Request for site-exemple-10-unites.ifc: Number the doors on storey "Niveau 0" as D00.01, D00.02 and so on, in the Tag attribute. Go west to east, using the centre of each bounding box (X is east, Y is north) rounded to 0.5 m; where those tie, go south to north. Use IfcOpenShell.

First a look at what the model holds.

```python
import ifcopenshell
import ifcopenshell.util.element
import ifcopenshell.util.placement

model = ifcopenshell.open("site-exemple-10-unites.ifc")
print(model.schema)
storey = next(s for s in model.by_type("IfcBuildingStorey") if s.Name == "Niveau 0")
doors = [e for e in ifcopenshell.util.element.get_decomposition(storey) if e.is_a("IfcDoor")]
for e in sorted(doors, key=lambda e: e.id()):
    origin = ifcopenshell.util.placement.get_local_placement(e.ObjectPlacement)[:3, 3]
    print(e.id(), e.Tag, e.Name, origin.round(2) + 0.0, sep=" | ")
```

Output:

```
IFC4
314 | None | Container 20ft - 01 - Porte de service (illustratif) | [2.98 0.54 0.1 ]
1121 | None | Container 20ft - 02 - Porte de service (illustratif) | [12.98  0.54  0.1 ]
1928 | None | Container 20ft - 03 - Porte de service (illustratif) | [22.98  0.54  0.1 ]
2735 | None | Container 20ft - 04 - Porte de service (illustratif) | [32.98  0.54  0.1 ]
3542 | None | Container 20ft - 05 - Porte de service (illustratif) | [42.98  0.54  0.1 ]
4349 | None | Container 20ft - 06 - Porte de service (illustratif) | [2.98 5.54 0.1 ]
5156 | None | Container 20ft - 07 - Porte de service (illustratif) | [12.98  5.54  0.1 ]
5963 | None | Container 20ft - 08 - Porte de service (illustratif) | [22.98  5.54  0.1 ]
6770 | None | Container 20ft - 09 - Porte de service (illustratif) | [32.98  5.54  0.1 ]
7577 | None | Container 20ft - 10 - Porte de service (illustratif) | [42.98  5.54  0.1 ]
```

```python
import ifcopenshell
import ifcopenshell.geom
import ifcopenshell.util.element
import ifcopenshell.util.shape

model = ifcopenshell.open("site-exemple-10-unites.ifc")
settings = ifcopenshell.geom.settings()
settings.set("use-world-coords", True)


def centre(element):
    shape = ifcopenshell.geom.create_shape(settings, element)
    return ifcopenshell.util.shape.get_bbox_centroid(shape.geometry)


storey = next(s for s in model.by_type("IfcBuildingStorey") if s.Name == "Niveau 0")
doors = [e for e in ifcopenshell.util.element.get_decomposition(storey) if e.is_a("IfcDoor")]

# Insertion points can sit at a corner or the storey origin, so sort by the geometry (in metres).
centres = {e: centre(e) for e in doors}
doors.sort(key=lambda e: (round(centres[e][0] / 0.5), centres[e][1]))

for i, e in enumerate(doors, start=1):
    number = f"D00.{i:02d}"
    e.Tag = number
    print(e.id(), number)

model.write("site-exemple-10-unites_edited.ifc")
```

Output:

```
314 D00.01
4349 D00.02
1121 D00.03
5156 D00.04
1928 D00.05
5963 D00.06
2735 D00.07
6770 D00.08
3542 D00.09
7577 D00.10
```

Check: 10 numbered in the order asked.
